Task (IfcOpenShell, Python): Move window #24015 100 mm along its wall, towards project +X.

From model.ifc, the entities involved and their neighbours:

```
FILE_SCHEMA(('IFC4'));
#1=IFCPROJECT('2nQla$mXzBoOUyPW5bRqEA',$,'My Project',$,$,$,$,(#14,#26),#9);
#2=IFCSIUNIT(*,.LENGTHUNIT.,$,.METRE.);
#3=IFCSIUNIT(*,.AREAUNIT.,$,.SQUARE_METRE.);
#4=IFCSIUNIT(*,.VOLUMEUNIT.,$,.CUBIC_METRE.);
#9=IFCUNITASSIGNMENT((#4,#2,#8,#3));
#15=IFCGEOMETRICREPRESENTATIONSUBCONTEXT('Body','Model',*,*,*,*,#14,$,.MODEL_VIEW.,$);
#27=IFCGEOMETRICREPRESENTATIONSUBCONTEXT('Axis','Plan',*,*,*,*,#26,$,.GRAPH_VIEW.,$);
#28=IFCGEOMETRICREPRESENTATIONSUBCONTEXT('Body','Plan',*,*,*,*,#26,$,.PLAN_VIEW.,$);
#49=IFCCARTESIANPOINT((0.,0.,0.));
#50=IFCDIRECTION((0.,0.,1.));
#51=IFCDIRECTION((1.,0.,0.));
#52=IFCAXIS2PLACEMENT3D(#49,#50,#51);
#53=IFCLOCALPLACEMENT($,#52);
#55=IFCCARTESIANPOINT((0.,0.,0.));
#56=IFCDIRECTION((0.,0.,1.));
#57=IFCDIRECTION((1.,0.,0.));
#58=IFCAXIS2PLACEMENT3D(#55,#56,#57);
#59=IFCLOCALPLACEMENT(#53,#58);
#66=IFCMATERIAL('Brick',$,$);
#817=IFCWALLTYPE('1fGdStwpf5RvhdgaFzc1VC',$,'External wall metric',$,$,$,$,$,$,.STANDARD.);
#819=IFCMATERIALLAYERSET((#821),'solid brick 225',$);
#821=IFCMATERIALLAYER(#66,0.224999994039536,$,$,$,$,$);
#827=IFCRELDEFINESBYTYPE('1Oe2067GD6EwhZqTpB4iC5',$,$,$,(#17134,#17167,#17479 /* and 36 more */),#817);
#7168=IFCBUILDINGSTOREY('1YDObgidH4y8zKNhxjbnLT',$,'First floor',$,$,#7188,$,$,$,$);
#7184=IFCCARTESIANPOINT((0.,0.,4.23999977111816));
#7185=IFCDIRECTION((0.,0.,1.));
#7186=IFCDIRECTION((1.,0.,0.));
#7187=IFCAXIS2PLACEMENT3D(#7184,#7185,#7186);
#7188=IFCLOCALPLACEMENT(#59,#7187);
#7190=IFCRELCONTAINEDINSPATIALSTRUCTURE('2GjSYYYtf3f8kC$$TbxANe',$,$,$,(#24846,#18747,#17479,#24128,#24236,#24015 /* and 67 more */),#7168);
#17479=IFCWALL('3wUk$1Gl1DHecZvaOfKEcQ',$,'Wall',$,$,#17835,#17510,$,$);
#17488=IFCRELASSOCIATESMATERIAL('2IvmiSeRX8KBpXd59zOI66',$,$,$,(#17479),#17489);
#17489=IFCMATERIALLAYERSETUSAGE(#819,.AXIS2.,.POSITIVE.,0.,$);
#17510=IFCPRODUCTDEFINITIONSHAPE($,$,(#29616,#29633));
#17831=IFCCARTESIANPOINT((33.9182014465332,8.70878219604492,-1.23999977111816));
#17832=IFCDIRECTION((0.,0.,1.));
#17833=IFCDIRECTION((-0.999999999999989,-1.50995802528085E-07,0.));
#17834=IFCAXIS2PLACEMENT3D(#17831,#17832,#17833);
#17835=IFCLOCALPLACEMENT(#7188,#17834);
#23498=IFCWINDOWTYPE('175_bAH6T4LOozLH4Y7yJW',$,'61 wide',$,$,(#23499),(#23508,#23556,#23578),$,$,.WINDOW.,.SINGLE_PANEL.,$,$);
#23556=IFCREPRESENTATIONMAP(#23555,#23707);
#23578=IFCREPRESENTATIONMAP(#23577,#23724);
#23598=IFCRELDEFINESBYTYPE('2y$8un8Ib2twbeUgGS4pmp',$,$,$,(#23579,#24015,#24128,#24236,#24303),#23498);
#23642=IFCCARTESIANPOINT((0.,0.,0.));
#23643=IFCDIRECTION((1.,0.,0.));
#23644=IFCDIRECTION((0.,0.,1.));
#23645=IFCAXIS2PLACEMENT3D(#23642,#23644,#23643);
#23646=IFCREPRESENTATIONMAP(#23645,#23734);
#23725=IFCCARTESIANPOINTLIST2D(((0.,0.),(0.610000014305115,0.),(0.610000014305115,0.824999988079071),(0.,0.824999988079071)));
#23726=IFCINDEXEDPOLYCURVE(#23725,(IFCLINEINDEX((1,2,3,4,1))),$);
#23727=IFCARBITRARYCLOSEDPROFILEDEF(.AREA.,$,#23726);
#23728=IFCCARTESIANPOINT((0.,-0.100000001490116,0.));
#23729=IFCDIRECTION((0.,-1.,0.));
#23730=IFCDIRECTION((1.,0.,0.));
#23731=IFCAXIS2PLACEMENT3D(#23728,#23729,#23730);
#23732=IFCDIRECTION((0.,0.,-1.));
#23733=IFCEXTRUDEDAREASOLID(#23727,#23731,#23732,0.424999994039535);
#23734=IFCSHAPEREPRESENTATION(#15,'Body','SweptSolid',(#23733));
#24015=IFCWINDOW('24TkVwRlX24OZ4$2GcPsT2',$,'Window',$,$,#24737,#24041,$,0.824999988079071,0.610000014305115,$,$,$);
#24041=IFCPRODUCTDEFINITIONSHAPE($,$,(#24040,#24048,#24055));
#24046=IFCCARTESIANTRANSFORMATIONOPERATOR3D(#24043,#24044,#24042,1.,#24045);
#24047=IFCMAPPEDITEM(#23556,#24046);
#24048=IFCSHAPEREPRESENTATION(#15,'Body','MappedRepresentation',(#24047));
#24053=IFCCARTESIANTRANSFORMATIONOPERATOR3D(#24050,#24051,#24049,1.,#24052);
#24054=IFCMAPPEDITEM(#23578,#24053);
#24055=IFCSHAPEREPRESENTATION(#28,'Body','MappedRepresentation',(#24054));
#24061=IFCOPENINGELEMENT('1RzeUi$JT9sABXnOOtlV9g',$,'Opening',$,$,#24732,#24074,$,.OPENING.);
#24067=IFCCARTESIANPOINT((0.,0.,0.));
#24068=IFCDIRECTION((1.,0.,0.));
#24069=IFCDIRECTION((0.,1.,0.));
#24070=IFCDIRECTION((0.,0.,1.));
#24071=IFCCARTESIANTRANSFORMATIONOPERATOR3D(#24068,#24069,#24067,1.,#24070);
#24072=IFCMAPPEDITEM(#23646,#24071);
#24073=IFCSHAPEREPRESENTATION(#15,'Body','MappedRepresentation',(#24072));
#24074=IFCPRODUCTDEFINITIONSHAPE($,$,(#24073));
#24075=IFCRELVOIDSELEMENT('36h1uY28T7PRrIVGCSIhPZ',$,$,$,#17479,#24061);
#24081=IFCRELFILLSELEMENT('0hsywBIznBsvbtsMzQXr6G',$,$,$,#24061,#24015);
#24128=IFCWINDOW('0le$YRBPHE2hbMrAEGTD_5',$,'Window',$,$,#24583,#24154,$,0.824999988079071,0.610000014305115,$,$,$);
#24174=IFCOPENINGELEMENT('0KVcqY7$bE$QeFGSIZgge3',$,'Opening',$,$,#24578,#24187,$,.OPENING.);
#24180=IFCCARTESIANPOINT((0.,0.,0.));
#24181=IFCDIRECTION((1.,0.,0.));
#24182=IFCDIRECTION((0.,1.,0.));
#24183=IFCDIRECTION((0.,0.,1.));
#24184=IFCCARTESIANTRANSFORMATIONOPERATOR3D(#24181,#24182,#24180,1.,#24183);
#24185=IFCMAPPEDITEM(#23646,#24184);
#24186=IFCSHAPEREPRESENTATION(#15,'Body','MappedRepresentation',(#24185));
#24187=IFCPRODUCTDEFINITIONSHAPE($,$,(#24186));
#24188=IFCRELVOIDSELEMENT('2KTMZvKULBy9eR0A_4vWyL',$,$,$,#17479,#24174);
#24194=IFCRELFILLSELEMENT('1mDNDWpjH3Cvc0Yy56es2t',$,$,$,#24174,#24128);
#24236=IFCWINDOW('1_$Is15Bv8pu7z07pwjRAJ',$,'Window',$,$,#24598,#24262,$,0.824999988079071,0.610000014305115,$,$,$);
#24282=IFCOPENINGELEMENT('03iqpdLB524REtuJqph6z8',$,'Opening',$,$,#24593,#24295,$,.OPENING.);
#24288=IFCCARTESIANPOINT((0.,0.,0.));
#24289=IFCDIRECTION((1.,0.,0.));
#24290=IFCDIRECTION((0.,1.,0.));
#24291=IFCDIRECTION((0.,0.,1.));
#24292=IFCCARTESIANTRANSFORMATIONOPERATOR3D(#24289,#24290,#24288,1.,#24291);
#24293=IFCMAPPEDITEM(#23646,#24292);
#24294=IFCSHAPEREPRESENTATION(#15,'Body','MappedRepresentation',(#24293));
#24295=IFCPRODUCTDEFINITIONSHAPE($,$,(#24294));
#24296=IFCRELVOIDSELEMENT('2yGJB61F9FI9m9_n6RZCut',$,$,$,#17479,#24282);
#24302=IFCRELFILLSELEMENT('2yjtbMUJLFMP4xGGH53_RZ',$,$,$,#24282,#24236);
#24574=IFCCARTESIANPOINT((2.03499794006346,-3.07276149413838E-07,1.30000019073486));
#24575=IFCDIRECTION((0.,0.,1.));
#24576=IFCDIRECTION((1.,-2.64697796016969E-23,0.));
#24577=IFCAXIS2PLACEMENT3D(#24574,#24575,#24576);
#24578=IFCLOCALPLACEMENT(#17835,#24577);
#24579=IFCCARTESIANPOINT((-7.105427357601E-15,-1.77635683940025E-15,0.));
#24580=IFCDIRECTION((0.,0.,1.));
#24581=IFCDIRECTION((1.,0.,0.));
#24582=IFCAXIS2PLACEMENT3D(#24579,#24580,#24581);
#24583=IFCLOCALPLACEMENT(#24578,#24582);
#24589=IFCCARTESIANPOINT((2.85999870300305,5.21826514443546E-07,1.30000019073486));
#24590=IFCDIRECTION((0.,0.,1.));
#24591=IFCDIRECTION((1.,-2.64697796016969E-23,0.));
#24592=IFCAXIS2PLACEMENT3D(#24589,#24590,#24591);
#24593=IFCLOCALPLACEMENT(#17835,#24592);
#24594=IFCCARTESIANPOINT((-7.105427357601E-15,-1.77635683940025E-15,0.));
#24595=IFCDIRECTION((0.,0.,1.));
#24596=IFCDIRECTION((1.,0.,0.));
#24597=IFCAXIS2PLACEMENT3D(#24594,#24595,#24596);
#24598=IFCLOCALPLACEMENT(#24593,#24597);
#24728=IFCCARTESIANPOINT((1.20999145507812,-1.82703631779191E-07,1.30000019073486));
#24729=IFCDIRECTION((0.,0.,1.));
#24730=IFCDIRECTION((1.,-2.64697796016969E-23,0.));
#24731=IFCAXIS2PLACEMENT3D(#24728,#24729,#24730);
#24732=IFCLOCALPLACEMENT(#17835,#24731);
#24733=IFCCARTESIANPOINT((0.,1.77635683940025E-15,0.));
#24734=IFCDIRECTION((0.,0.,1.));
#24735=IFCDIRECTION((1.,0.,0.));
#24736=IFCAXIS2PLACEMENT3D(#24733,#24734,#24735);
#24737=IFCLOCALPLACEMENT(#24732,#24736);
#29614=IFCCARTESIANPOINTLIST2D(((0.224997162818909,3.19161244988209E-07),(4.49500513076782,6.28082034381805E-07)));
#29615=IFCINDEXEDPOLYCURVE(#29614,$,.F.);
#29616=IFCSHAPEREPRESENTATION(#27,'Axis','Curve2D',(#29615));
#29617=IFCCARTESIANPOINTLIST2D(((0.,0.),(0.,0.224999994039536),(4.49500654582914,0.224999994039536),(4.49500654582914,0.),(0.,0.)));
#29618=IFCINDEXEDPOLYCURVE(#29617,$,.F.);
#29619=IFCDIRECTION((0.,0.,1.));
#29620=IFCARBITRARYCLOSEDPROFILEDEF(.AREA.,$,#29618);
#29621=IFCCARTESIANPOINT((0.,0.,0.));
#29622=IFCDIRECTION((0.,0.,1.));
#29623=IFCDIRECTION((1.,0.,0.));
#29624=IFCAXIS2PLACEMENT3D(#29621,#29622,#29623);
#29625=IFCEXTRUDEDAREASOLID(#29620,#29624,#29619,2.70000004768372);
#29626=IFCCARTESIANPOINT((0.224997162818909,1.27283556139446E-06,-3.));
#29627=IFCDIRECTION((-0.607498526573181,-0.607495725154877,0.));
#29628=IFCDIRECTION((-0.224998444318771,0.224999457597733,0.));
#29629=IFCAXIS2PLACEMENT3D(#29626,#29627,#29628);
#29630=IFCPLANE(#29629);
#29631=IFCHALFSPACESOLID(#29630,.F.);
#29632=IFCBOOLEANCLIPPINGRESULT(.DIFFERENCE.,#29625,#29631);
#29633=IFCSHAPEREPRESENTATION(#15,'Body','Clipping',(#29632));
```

```python
import ifcopenshell
import ifcopenshell.api.geometry
import ifcopenshell.util.placement
import ifcopenshell.util.unit

model = ifcopenshell.open("model.ifc")
unit_scale = ifcopenshell.util.unit.calculate_unit_scale(model)

window = model.by_guid("24TkVwRlX24OZ4$2GcPsT2")
opening = window.FillsVoids[0].RelatingOpeningElement
wall = opening.VoidsElements[0].RelatingBuildingElement

wall_matrix = ifcopenshell.util.placement.get_local_placement(wall.ObjectPlacement)
shift = wall_matrix[:3, 0] * -0.1 / unit_scale
before = ifcopenshell.util.placement.get_local_placement(window.ObjectPlacement)[:3, 3].copy()

# The window is placed relative to its opening, so it follows when the opening moves.
matrix = ifcopenshell.util.placement.get_local_placement(opening.ObjectPlacement)
matrix[:3, 3] += shift
ifcopenshell.api.geometry.edit_object_placement(
    model, product=opening, matrix=matrix, is_si=False, should_transform_children=True
)

after = ifcopenshell.util.placement.get_local_placement(window.ObjectPlacement)[:3, 3]
print("window moved by", (after - before).round(3) + 0.0)

model.write("model_v2.ifc")
```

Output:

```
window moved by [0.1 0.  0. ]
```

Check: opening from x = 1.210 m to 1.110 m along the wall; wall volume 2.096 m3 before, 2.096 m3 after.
